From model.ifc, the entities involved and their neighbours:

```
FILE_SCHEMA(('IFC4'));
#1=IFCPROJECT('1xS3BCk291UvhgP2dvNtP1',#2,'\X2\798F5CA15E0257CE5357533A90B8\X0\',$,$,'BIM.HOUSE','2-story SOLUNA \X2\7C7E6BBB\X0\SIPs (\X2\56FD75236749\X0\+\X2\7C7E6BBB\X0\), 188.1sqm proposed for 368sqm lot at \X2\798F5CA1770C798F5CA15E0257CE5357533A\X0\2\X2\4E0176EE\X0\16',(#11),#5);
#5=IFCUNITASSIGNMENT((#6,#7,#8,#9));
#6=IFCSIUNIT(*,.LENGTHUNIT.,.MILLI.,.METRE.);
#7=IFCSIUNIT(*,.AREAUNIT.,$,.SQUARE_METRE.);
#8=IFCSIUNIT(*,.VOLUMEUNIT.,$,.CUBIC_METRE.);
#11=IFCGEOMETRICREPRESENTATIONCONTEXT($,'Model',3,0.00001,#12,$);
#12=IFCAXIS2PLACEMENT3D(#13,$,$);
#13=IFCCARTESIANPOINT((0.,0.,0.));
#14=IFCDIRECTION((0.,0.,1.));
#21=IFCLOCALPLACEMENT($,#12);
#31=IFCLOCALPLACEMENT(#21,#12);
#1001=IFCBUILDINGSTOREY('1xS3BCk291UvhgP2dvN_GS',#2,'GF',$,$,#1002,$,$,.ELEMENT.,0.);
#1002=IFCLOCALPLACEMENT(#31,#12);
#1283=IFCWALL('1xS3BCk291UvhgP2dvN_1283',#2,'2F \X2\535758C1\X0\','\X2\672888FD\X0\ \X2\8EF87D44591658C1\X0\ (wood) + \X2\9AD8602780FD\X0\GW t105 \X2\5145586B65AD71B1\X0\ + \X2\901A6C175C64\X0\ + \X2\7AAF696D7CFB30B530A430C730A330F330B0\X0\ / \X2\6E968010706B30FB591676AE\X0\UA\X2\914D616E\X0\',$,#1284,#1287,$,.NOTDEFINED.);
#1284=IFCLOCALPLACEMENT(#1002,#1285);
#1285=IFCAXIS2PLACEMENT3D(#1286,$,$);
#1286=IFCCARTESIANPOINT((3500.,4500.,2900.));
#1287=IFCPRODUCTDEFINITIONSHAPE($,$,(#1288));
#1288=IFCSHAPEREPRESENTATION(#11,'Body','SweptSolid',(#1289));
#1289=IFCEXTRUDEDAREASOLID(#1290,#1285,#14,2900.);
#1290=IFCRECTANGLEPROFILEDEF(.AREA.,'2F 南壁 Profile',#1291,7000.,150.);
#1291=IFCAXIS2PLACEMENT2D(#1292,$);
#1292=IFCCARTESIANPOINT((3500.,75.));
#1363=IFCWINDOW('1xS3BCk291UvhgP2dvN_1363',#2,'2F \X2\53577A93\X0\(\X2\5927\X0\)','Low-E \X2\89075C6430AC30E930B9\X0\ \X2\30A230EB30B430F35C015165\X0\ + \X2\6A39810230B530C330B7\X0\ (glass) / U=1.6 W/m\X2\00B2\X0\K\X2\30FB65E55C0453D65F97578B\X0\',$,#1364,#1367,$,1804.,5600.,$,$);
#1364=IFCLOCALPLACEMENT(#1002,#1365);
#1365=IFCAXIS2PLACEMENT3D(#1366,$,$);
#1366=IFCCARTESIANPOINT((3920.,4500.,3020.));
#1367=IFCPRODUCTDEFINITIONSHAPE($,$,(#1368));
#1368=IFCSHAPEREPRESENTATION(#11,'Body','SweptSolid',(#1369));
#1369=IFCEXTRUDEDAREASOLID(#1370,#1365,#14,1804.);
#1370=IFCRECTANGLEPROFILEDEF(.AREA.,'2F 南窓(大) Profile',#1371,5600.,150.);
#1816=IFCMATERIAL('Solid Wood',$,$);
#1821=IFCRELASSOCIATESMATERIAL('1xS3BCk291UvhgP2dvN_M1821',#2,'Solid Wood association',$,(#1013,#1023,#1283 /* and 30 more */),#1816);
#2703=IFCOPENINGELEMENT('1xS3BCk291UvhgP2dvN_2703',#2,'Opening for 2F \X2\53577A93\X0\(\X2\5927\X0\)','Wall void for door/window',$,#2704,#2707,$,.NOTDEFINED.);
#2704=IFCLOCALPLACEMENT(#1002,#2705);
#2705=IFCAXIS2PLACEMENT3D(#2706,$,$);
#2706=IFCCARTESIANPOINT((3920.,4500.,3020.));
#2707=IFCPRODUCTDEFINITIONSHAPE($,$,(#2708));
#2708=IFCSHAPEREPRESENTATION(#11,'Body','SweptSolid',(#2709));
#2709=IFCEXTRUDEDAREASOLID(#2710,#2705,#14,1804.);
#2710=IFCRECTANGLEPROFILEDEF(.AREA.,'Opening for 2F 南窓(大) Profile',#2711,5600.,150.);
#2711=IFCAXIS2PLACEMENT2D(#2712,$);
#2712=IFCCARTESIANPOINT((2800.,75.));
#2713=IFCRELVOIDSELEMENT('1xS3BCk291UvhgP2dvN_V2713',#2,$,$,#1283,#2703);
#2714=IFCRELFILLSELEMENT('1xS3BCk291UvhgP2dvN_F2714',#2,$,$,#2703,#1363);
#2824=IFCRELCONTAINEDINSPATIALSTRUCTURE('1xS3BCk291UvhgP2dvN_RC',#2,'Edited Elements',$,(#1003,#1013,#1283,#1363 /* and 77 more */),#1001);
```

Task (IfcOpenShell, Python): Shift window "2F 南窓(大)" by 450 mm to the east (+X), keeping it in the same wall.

```python
import ifcopenshell
import ifcopenshell.api.geometry
import ifcopenshell.util.placement

model = ifcopenshell.open("model.ifc")

window = model.by_guid("1xS3BCk291UvhgP2dvN_1363")
opening = window.FillsVoids[0].RelatingOpeningElement
wall = opening.VoidsElements[0].RelatingBuildingElement

wall_matrix = ifcopenshell.util.placement.get_local_placement(wall.ObjectPlacement)
shift = wall_matrix[:3, 0] * 450.0
before = ifcopenshell.util.placement.get_local_placement(window.ObjectPlacement)[:3, 3].copy()

# The window is not placed relative to its opening, so move both.
for product in (opening, window):
    matrix = ifcopenshell.util.placement.get_local_placement(product.ObjectPlacement)
    matrix[:3, 3] += shift
    ifcopenshell.api.geometry.edit_object_placement(model, product=product, matrix=matrix, is_si=False)

after = ifcopenshell.util.placement.get_local_placement(window.ObjectPlacement)[:3, 3]
print("window moved by", (after - before).round(3) + 0.0)

model.write("model_edited.ifc")
```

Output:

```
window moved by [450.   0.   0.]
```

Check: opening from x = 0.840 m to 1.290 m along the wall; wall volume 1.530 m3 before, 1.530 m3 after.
